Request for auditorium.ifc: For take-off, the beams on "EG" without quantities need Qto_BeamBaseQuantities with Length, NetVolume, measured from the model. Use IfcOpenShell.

First a look at what the model holds.

```python
import ifcopenshell
import ifcopenshell.util.element
import ifcopenshell.util.unit

model = ifcopenshell.open("auditorium.ifc")
print(model.schema)
for unit_type in ("LENGTHUNIT", "AREAUNIT", "VOLUMEUNIT"):
    print(unit_type, ifcopenshell.util.unit.calculate_unit_scale(model, unit_type))
storey = next(s for s in model.by_type("IfcBuildingStorey") if s.Name == "EG")
beams = [e for e in ifcopenshell.util.element.get_decomposition(storey) if e.is_a("IfcBeam")]
for e in sorted(beams, key=lambda e: e.id()):
    print(e.id(), e.is_a(), e.Name, list(ifcopenshell.util.element.get_psets(e, qtos_only=True)), sep=" | ")
```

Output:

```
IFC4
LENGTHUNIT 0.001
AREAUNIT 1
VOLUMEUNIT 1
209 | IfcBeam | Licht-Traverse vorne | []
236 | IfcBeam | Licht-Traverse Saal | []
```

```python
import ifcopenshell
import ifcopenshell.api.pset
import ifcopenshell.geom
import ifcopenshell.util.element
import ifcopenshell.util.shape
import ifcopenshell.util.unit

model = ifcopenshell.open("auditorium.ifc")
unit_scale = ifcopenshell.util.unit.calculate_unit_scale(model)
volume_scale = ifcopenshell.util.unit.calculate_unit_scale(model, "VOLUMEUNIT")
settings = ifcopenshell.geom.settings()

storey = next(s for s in model.by_type("IfcBuildingStorey") if s.Name == "EG")
beams = [e for e in ifcopenshell.util.element.get_decomposition(storey) if e.is_a("IfcBeam")]

for e in sorted(beams, key=lambda e: e.id()):
    if ifcopenshell.util.element.get_psets(e, qtos_only=True, should_inherit=False):
        continue
    # Geometry comes back in metres, in the element's own axes.
    shape = ifcopenshell.geom.create_shape(settings, e)
    values = {
        "Length": ifcopenshell.util.shape.get_max_xyz(shape.geometry) / unit_scale,
        "NetVolume": ifcopenshell.util.shape.get_volume(shape.geometry) / volume_scale,
    }
    qto = ifcopenshell.api.pset.add_qto(model, product=e, name="Qto_BeamBaseQuantities")
    ifcopenshell.api.pset.edit_qto(model, qto=qto, properties=values)
    print(e.id(), {k: round(v, 3) for k, v in values.items()})

model.write("auditorium-out.ifc")
```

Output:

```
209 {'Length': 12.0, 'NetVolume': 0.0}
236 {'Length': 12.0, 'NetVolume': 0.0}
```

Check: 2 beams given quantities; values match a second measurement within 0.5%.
